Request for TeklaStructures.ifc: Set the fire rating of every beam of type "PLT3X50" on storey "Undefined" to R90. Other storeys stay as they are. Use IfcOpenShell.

First a look at what the model holds.

```python
import ifcopenshell
import ifcopenshell.util.element

model = ifcopenshell.open("TeklaStructures.ifc")
print(model.schema)
storey = next(s for s in model.by_type("IfcBuildingStorey") if s.Name == "Undefined")
beams = [e for e in ifcopenshell.util.element.get_decomposition(storey) if e.is_a("IfcBeam")]
seen = {}
for e in beams:
    element_type = ifcopenshell.util.element.get_type(e)
    key = (element_type.Name if element_type != e and element_type else None, ifcopenshell.util.element.get_pset(e, "Pset_BeamCommon", "FireRating"))
    seen[key] = seen.get(key, 0) + 1
for (name, value), count in sorted(seen.items(), key=str):
    print(count, "x", name, "|", value)
```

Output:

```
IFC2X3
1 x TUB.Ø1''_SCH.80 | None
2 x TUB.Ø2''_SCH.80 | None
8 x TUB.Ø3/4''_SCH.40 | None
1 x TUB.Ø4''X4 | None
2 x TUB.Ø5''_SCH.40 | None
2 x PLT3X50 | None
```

```python
import ifcopenshell
import ifcopenshell.api.pset
import ifcopenshell.util.element

model = ifcopenshell.open("TeklaStructures.ifc")

storey = next(s for s in model.by_type("IfcBuildingStorey") if s.Name == "Undefined")
beams = [e for e in ifcopenshell.util.element.get_decomposition(storey) if e.is_a("IfcBeam")]

count = 0
for e in beams:
    element_type = ifcopenshell.util.element.get_type(e)
    if element_type in (None, e) or element_type.Name != "PLT3X50":
        continue
    # add_pset returns the element's existing set when there is one.
    pset = ifcopenshell.api.pset.add_pset(model, product=e, name="Pset_BeamCommon")
    ifcopenshell.api.pset.edit_pset(model, pset=pset, properties={"FireRating": "R90"})
    count += 1

print(count, "beams updated")

model.write("TeklaStructures_updated.ifc")
```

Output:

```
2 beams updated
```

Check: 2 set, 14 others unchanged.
